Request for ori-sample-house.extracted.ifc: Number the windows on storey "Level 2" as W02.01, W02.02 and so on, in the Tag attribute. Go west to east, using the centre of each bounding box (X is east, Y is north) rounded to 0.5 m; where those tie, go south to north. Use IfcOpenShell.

First a look at what the model holds.

```python
import ifcopenshell
import ifcopenshell.util.element
import ifcopenshell.util.placement

model = ifcopenshell.open("ori-sample-house.extracted.ifc")
print(model.schema)
storey = next(s for s in model.by_type("IfcBuildingStorey") if s.Name == "Level 2")
windows = [e for e in ifcopenshell.util.element.get_decomposition(storey) if e.is_a("IfcWindow")]
for e in sorted(windows, key=lambda e: e.id()):
    origin = ifcopenshell.util.placement.get_local_placement(e.ObjectPlacement)[:3, 3]
    print(e.id(), e.Tag, e.Name, origin.round(2) + 0.0, sep=" | ")
```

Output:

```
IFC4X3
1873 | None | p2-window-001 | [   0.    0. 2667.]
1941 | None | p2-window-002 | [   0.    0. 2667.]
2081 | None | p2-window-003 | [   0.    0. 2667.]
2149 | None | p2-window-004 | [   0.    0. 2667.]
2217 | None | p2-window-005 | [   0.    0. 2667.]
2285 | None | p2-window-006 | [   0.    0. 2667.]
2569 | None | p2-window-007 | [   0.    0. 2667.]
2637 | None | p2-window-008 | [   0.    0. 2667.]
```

```python
import ifcopenshell
import ifcopenshell.geom
import ifcopenshell.util.element
import ifcopenshell.util.shape

model = ifcopenshell.open("ori-sample-house.extracted.ifc")
settings = ifcopenshell.geom.settings()
settings.set("use-world-coords", True)


def centre(element):
    shape = ifcopenshell.geom.create_shape(settings, element)
    return ifcopenshell.util.shape.get_bbox_centroid(shape.geometry)


storey = next(s for s in model.by_type("IfcBuildingStorey") if s.Name == "Level 2")
windows = [e for e in ifcopenshell.util.element.get_decomposition(storey) if e.is_a("IfcWindow")]

# Insertion points can sit at a corner or the storey origin, so sort by the geometry (in metres).
centres = {e: centre(e) for e in windows}
windows.sort(key=lambda e: (round(centres[e][0] / 0.5), centres[e][1]))

for i, e in enumerate(windows, start=1):
    number = f"W02.{i:02d}"
    e.Tag = number
    print(e.id(), number)

model.write("ori-sample-house.extracted_v2.ifc")
```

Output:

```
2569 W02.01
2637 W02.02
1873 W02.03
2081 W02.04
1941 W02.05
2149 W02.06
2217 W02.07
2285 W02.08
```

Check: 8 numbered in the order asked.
